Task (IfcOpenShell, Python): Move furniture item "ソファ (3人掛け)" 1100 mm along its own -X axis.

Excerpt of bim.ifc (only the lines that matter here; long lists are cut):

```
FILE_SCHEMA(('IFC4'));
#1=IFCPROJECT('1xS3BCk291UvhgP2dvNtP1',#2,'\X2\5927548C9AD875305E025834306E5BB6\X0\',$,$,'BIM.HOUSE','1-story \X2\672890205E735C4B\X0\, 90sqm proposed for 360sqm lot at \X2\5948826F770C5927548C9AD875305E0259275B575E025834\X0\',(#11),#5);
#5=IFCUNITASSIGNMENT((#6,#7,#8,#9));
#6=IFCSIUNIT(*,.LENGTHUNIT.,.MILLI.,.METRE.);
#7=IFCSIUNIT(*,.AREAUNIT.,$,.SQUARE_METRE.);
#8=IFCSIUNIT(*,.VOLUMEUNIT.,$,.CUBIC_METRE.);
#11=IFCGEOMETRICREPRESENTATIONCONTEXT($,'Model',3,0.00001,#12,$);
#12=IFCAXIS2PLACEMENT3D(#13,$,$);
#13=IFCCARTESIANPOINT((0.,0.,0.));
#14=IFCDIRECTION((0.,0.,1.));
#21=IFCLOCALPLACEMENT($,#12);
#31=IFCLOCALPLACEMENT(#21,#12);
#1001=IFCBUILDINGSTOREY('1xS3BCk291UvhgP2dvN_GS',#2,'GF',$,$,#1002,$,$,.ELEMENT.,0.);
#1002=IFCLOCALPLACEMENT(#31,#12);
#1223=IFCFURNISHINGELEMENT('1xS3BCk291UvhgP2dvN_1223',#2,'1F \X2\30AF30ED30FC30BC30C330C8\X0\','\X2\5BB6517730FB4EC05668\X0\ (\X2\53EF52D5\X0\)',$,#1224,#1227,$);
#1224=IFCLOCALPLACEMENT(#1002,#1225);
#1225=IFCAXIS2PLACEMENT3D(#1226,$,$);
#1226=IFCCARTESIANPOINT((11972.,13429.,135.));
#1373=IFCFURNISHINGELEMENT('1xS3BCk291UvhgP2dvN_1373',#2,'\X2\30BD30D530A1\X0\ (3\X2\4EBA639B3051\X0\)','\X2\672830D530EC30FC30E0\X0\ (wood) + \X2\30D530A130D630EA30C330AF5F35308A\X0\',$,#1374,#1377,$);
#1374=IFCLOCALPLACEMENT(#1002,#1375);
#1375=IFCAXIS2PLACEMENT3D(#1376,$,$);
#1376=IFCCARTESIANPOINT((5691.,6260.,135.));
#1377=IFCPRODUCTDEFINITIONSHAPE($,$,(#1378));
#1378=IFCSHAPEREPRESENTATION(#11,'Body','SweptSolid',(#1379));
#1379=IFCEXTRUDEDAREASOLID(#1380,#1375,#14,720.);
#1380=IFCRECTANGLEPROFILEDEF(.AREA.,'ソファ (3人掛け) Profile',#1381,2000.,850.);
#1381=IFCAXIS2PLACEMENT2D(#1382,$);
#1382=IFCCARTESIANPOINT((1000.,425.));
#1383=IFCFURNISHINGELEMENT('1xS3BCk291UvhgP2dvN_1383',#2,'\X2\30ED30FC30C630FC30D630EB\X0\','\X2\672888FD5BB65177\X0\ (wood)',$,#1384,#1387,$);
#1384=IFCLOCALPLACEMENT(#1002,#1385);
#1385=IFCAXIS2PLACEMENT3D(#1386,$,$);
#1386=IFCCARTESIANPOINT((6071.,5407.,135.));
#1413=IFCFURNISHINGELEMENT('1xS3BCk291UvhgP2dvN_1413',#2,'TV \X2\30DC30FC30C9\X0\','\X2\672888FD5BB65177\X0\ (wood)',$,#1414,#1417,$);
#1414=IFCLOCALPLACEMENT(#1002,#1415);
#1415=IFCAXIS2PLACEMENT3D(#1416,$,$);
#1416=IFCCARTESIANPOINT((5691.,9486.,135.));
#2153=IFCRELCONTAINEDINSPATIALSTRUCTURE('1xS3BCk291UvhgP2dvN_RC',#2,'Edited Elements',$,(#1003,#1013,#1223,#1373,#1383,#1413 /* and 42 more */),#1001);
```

```python
import ifcopenshell
import ifcopenshell.api.geometry
import ifcopenshell.util.placement

model = ifcopenshell.open("bim.ifc")

item = model.by_guid("1xS3BCk291UvhgP2dvN_1373")
matrix = ifcopenshell.util.placement.get_local_placement(item.ObjectPlacement)
matrix[:3, 3] -= matrix[:3, 0] * 1100.0
ifcopenshell.api.geometry.edit_object_placement(model, product=item, matrix=matrix, is_si=False)

print(ifcopenshell.util.placement.get_local_placement(item.ObjectPlacement).round(3) + 0.0)

model.write("bim_v2.ifc")
```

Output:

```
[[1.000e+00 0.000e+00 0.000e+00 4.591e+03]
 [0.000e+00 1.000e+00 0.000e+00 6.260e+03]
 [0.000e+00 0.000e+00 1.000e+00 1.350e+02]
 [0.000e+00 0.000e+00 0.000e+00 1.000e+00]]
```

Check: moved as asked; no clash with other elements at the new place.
